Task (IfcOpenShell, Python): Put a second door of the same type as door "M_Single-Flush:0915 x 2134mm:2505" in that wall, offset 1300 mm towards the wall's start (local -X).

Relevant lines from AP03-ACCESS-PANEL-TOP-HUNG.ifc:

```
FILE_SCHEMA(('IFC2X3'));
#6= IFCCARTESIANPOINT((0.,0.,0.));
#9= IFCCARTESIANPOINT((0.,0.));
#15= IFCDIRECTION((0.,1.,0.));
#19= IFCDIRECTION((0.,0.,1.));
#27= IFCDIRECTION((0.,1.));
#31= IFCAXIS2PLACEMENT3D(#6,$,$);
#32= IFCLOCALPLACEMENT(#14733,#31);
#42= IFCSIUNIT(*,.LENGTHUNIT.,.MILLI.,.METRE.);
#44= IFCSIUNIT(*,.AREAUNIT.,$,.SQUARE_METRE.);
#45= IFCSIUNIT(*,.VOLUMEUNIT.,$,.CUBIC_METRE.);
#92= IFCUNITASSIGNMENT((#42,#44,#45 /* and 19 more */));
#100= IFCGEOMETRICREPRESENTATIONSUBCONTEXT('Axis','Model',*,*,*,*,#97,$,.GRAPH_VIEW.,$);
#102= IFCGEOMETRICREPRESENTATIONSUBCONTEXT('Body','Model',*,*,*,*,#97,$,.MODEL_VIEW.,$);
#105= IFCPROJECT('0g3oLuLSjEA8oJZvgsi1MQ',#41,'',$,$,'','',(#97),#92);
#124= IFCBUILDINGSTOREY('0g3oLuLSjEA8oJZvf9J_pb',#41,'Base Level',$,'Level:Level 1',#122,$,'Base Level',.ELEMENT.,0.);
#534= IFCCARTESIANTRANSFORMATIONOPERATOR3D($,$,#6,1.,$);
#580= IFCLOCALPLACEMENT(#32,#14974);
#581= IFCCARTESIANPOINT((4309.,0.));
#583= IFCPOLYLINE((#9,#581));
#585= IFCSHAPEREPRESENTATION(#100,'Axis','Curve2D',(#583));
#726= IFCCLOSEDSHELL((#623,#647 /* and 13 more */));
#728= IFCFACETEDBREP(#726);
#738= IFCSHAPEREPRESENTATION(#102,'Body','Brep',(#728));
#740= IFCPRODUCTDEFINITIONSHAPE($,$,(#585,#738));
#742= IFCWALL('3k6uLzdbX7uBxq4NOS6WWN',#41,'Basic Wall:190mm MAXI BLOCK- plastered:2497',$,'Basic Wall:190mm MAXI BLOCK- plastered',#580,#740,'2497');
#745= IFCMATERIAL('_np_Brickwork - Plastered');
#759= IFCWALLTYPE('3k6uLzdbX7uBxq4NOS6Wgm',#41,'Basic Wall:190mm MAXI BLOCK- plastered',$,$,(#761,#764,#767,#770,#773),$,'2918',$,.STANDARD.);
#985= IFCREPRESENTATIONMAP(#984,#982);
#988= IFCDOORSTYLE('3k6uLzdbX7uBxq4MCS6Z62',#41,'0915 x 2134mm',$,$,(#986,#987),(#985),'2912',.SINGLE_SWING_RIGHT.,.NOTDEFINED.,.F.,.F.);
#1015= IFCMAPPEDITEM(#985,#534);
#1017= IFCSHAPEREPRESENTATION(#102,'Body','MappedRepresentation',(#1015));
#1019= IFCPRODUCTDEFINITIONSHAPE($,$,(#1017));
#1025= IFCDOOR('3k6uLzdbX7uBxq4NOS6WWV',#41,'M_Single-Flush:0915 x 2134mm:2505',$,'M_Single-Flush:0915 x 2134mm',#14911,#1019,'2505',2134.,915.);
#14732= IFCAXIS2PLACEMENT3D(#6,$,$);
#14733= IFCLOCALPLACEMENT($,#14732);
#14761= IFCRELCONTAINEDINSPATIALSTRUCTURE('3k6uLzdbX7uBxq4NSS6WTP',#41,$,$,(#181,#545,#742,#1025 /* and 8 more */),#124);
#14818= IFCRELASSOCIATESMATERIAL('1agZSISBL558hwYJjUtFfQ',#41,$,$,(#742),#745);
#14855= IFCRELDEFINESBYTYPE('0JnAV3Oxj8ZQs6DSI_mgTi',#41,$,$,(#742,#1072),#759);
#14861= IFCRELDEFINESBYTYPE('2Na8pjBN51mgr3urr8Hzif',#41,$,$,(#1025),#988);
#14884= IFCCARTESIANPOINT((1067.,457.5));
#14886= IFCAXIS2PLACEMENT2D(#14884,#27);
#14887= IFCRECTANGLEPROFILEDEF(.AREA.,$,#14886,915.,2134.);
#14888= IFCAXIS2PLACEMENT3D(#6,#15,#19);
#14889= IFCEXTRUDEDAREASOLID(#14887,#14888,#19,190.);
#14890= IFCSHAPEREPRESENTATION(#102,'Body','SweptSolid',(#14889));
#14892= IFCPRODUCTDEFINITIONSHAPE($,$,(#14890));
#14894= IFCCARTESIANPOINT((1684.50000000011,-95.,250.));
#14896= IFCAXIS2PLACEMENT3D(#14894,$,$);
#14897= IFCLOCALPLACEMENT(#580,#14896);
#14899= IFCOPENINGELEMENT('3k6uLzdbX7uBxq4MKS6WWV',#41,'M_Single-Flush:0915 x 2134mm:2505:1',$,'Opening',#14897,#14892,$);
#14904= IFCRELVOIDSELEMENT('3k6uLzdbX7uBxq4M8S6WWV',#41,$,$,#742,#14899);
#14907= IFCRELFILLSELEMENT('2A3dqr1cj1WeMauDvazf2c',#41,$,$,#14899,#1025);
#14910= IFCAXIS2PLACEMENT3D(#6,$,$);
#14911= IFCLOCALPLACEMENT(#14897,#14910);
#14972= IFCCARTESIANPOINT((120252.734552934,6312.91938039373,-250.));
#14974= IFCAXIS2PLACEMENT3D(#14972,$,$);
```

```python
import ifcopenshell
import ifcopenshell.api.feature
import ifcopenshell.api.geometry
import ifcopenshell.api.root
import ifcopenshell.geom
import ifcopenshell.util.element
import ifcopenshell.util.placement
import ifcopenshell.util.shape
import ifcopenshell.util.unit

model = ifcopenshell.open("AP03-ACCESS-PANEL-TOP-HUNG.ifc")
unit_scale = ifcopenshell.util.unit.calculate_unit_scale(model)
settings = ifcopenshell.geom.settings()


def volume(element):
    """Net volume in cubic metres, openings subtracted."""
    shape = ifcopenshell.geom.create_shape(settings, element)
    return ifcopenshell.util.shape.get_volume(shape.geometry)


def reuse_history(source, copy):
    """copy_class also copies each property set's owner history, people and application; keep the originals."""
    for rel in copy.IsDefinedBy:
        if rel.is_a("IfcRelDefinesByProperties") and (history := rel.RelatingPropertyDefinition.OwnerHistory):
            rel.RelatingPropertyDefinition.OwnerHistory = source.OwnerHistory
            ifcopenshell.util.element.remove_deep2(model, history)


door = model.by_id(1025)
opening = door.FillsVoids[0].RelatingOpeningElement
wall = opening.VoidsElements[0].RelatingBuildingElement
before = volume(wall)
shift = ifcopenshell.util.placement.get_local_placement(wall.ObjectPlacement)[:3, 0] * -1.3 / unit_scale

# copy_class copies the void relationship, type, container and properties, but no geometry.
new_opening = ifcopenshell.api.root.copy_class(model, product=opening)
new_opening.Representation = ifcopenshell.util.element.copy_deep(
    model, opening.Representation, exclude=["IfcGeometricRepresentationContext", "IfcRepresentationMap"]
)
new_opening.Name = "M_Single-Flush:0915 x 2134mm"
new_door = ifcopenshell.api.root.copy_class(model, product=door)
new_door.Representation = ifcopenshell.util.element.copy_deep(
    model, door.Representation, exclude=["IfcGeometricRepresentationContext", "IfcRepresentationMap"]
)
new_door.Name = "M_Single-Flush:0915 x 2134mm"
new_door.Tag = None
reuse_history(door, new_door)
fills = ifcopenshell.api.feature.add_filling(model, opening=new_opening, element=new_door)
fills.OwnerHistory = new_door.OwnerHistory  # required in IFC2X3

for old, new in ((opening, new_opening), (door, new_door)):
    matrix = ifcopenshell.util.placement.get_local_placement(old.ObjectPlacement)
    matrix[:3, 3] += shift
    ifcopenshell.api.geometry.edit_object_placement(model, product=new, matrix=matrix, is_si=False)

after = volume(wall)

print(f"wall volume {before:.3f} -> {after:.3f} m3")

model.write("AP03-ACCESS-PANEL-TOP-HUNG_v2.ifc")
```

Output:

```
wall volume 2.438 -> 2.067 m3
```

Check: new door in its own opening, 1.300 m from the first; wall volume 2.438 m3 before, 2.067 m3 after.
